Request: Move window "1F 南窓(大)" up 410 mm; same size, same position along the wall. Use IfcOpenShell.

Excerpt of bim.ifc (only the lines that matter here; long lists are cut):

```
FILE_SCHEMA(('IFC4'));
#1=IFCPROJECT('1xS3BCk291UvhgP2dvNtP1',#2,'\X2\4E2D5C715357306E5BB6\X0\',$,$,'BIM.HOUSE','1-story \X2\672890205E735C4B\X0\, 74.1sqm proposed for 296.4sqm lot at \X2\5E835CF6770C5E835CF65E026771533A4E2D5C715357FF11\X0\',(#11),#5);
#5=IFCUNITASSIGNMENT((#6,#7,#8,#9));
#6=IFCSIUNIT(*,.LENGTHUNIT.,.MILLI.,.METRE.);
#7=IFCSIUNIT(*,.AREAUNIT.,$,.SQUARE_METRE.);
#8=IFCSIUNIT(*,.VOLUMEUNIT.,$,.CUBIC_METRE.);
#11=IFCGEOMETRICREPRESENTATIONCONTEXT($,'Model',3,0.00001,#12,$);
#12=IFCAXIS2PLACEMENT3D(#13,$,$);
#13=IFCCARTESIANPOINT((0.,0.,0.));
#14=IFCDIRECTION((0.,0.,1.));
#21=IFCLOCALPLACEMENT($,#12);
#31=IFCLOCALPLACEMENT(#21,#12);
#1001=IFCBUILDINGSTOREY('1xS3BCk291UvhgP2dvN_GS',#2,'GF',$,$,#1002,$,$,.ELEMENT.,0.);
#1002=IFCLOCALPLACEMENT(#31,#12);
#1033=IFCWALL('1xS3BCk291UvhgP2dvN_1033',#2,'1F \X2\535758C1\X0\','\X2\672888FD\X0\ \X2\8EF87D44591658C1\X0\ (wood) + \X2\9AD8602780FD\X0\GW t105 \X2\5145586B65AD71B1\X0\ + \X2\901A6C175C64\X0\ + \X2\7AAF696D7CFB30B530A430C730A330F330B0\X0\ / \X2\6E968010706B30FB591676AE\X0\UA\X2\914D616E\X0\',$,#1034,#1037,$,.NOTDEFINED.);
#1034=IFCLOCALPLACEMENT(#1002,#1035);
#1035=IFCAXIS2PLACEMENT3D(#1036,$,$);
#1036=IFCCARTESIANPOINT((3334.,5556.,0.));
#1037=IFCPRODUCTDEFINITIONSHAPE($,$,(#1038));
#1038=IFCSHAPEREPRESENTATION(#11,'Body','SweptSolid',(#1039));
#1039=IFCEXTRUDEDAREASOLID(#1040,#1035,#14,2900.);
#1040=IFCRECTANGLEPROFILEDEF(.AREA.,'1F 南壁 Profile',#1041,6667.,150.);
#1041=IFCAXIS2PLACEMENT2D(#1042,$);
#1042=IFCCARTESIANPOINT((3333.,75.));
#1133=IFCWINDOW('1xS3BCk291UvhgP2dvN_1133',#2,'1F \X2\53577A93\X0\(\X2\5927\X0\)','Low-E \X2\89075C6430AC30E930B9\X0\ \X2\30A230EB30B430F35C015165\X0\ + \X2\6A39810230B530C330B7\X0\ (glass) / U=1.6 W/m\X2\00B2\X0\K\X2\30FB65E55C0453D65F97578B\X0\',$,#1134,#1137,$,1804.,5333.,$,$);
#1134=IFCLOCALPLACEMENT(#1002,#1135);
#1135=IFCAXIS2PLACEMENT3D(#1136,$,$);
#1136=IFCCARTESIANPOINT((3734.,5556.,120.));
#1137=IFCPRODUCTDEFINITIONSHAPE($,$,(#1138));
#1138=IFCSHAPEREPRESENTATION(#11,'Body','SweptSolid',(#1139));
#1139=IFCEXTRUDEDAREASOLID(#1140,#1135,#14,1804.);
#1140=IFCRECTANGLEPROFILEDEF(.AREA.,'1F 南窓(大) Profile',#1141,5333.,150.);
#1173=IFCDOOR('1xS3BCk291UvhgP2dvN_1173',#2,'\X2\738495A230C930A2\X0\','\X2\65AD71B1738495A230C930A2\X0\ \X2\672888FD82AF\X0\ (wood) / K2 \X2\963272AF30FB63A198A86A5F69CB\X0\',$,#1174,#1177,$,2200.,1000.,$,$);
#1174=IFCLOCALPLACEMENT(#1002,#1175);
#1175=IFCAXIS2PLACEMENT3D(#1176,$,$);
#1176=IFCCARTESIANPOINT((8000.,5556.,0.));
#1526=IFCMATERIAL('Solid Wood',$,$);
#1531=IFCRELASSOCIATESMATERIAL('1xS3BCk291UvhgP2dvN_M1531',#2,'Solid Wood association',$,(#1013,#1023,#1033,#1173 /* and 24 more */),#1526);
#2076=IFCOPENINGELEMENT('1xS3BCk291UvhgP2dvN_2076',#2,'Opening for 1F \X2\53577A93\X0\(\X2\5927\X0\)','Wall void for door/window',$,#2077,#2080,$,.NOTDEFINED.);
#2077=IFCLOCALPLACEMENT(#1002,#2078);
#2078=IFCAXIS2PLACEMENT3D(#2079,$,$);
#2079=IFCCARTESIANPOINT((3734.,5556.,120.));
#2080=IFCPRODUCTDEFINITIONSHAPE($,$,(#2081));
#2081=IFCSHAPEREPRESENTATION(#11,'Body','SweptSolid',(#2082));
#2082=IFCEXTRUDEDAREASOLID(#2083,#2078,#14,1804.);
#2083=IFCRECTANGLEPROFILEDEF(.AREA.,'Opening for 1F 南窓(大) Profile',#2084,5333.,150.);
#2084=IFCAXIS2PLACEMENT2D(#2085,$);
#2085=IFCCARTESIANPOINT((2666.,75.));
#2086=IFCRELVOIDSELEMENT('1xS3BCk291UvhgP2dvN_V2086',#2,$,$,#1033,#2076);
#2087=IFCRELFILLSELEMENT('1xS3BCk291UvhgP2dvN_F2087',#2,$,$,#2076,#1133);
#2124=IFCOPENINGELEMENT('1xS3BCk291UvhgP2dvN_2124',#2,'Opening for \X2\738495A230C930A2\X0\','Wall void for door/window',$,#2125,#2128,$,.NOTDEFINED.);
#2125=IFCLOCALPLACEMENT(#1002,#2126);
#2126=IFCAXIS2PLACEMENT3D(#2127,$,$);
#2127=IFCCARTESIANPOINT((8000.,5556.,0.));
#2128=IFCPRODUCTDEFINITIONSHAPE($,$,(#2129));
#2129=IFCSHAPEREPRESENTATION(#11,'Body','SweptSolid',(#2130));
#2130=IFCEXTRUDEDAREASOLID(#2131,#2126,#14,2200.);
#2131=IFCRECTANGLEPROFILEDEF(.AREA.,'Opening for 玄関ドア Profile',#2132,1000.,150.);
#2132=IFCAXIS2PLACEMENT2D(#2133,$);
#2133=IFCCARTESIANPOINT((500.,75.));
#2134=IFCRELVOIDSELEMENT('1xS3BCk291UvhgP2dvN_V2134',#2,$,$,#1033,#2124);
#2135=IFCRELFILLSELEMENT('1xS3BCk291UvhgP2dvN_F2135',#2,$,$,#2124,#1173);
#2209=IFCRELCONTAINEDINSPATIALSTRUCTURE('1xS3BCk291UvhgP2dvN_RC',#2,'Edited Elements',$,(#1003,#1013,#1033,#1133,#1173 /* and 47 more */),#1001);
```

```python
import numpy as np
import ifcopenshell
import ifcopenshell.api.geometry
import ifcopenshell.util.placement
import ifcopenshell.util.unit

model = ifcopenshell.open("bim.ifc")
unit_scale = ifcopenshell.util.unit.calculate_unit_scale(model)

window = model.by_id(1133)
opening = window.FillsVoids[0].RelatingOpeningElement
dz = 410.0

shift = np.array([0.0, 0.0, dz])
# The window is not placed relative to its opening, so move both.
for product in (opening, window):
    matrix = ifcopenshell.util.placement.get_local_placement(product.ObjectPlacement)
    matrix[:3, 3] += shift
    ifcopenshell.api.geometry.edit_object_placement(model, product=product, matrix=matrix, is_si=False)

print(f"moved by {dz * unit_scale:+.3f} m")

model.write("bim_v2.ifc")
```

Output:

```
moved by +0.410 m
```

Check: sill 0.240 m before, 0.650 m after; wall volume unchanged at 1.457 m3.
